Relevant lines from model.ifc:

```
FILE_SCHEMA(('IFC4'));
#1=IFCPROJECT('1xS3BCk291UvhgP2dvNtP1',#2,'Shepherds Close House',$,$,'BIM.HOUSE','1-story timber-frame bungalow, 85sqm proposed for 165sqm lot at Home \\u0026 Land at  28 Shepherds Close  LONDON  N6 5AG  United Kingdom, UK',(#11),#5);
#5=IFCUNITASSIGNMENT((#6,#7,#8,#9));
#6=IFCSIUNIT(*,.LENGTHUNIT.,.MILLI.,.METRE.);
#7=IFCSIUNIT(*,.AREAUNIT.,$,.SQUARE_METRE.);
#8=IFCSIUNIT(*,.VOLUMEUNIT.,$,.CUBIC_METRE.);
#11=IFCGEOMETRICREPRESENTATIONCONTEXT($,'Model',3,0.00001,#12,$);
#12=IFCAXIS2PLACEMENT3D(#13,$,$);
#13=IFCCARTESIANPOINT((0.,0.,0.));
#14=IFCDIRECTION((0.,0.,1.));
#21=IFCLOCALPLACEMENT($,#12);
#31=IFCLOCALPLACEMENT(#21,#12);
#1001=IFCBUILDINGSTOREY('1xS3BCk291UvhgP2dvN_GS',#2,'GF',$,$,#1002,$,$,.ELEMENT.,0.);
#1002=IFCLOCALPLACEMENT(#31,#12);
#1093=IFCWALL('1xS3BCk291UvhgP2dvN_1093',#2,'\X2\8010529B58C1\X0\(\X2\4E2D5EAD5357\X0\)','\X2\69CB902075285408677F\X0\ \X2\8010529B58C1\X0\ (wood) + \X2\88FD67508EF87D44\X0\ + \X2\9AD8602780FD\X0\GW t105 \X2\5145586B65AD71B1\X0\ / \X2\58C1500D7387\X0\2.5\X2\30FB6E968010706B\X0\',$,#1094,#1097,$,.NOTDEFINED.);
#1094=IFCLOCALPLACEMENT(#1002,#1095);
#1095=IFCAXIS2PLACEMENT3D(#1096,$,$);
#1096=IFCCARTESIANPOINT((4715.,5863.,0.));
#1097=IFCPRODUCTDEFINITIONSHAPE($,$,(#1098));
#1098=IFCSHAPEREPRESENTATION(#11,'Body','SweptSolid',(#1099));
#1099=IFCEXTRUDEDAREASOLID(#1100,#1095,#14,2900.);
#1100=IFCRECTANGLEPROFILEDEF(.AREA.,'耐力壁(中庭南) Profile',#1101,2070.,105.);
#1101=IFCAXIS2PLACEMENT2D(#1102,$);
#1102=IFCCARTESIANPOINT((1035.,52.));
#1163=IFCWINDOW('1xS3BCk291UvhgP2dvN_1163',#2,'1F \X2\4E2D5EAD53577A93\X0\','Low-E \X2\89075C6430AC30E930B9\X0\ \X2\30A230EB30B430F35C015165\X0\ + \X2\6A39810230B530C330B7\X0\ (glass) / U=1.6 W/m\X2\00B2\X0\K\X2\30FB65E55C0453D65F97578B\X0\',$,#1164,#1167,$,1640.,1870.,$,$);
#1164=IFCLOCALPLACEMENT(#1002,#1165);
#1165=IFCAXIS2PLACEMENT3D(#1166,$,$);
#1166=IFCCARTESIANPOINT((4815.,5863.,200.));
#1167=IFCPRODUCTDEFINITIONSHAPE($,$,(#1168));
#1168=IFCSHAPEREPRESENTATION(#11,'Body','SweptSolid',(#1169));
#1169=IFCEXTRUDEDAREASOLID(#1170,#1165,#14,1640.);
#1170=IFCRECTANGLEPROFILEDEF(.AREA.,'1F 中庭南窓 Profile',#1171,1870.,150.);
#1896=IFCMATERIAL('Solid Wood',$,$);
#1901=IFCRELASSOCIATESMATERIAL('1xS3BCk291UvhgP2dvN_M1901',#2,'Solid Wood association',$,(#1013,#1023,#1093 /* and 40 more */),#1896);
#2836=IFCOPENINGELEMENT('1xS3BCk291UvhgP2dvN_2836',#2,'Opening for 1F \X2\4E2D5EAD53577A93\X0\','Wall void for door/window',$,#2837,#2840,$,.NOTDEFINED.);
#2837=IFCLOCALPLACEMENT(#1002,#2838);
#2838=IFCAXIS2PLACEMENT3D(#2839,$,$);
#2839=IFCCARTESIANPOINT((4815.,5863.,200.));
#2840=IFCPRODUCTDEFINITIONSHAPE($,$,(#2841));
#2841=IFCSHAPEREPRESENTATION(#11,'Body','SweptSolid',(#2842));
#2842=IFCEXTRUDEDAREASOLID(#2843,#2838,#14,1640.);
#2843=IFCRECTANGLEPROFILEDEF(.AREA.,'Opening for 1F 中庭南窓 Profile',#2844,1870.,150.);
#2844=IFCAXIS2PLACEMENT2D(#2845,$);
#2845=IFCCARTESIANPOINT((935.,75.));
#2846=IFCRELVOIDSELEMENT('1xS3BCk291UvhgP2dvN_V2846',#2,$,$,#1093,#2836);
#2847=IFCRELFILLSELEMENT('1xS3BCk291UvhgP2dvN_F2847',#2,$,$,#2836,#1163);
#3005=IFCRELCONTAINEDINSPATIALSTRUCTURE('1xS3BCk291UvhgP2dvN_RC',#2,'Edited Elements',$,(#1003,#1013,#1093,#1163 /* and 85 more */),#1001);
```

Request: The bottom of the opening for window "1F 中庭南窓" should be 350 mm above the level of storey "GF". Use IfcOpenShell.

```python
import numpy as np
import ifcopenshell
import ifcopenshell.api.geometry
import ifcopenshell.geom
import ifcopenshell.util.element
import ifcopenshell.util.placement
import ifcopenshell.util.shape
import ifcopenshell.util.unit

model = ifcopenshell.open("model.ifc")
unit_scale = ifcopenshell.util.unit.calculate_unit_scale(model)

window = model.by_guid("1xS3BCk291UvhgP2dvN_1163")
opening = window.FillsVoids[0].RelatingOpeningElement
storey = ifcopenshell.util.element.get_container(window, ifc_class="IfcBuildingStorey")
level = ifcopenshell.util.placement.get_local_placement(storey.ObjectPlacement)[2, 3]

# The opening's origin need not be at the sill, so measure its lowest point.
shape = ifcopenshell.geom.create_shape(ifcopenshell.geom.settings(), opening)
bottom = ifcopenshell.util.shape.get_shape_bottom_elevation(shape, shape.geometry) / unit_scale
dz = level + 0.35 / unit_scale - bottom

shift = np.array([0.0, 0.0, dz])
# The window is not placed relative to its opening, so move both.
for product in (opening, window):
    matrix = ifcopenshell.util.placement.get_local_placement(product.ObjectPlacement)
    matrix[:3, 3] += shift
    ifcopenshell.api.geometry.edit_object_placement(model, product=product, matrix=matrix, is_si=False)

print(f"moved by {dz * unit_scale:+.3f} m")

model.write("model_edited.ifc")
```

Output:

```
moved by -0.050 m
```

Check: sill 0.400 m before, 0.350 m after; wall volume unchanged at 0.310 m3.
